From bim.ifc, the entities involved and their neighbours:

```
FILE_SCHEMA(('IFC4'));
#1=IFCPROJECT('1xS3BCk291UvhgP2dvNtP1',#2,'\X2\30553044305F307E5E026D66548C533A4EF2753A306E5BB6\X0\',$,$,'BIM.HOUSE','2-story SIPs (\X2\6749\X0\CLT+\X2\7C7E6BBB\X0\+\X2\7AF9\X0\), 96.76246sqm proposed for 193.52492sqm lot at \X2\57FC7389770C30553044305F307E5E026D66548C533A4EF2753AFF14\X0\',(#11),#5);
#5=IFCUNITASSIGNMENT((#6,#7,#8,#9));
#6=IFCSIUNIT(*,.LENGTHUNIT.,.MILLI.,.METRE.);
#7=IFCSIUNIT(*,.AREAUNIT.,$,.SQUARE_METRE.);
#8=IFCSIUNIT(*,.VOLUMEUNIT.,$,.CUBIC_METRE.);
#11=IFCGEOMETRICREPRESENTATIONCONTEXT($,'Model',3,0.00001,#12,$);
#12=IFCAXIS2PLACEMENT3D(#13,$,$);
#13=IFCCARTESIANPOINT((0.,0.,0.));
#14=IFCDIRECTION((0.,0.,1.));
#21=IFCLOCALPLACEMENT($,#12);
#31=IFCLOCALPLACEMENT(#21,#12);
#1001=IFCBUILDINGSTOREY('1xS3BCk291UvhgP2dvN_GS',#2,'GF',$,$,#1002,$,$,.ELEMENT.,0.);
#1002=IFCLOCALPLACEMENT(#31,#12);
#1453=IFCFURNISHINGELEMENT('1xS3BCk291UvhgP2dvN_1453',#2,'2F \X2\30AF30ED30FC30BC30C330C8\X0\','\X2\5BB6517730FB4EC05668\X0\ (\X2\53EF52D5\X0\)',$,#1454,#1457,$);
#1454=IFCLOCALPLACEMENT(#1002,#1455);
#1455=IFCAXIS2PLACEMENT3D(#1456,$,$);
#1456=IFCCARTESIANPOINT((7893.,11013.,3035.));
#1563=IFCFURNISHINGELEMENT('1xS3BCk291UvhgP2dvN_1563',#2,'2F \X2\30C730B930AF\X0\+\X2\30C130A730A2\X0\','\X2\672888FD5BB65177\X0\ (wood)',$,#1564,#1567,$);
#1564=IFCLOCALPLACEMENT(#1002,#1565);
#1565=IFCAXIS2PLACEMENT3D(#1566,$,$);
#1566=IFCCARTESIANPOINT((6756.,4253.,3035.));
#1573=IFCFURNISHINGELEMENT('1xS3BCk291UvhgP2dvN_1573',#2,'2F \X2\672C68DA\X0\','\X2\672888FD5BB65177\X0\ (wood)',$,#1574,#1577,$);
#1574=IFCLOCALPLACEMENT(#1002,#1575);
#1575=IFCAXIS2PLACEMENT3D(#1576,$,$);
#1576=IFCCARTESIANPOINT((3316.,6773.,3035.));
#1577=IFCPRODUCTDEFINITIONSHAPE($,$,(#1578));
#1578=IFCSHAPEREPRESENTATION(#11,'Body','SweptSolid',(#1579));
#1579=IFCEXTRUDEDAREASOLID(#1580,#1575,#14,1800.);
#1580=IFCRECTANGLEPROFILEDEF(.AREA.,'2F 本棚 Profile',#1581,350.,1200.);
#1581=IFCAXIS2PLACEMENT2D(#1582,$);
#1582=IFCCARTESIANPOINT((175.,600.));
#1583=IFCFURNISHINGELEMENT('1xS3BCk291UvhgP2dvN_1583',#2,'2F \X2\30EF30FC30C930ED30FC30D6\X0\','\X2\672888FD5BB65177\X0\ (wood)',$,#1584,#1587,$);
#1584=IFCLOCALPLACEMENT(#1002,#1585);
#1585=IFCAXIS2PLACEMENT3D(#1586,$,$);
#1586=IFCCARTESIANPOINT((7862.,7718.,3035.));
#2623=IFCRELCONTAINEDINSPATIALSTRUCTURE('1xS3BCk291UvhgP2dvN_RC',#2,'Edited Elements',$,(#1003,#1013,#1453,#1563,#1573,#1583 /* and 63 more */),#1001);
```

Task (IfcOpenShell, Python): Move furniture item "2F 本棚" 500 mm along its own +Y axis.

```python
import ifcopenshell
import ifcopenshell.api.geometry
import ifcopenshell.util.placement
import ifcopenshell.util.unit

model = ifcopenshell.open("bim.ifc")
unit_scale = ifcopenshell.util.unit.calculate_unit_scale(model)

item = model.by_guid("1xS3BCk291UvhgP2dvN_1573")
matrix = ifcopenshell.util.placement.get_local_placement(item.ObjectPlacement)
matrix[:3, 3] += matrix[:3, 1] * 0.5 / unit_scale
ifcopenshell.api.geometry.edit_object_placement(model, product=item, matrix=matrix, is_si=False)

print(ifcopenshell.util.placement.get_local_placement(item.ObjectPlacement).round(3) + 0.0)

model.write("bim-out.ifc")
```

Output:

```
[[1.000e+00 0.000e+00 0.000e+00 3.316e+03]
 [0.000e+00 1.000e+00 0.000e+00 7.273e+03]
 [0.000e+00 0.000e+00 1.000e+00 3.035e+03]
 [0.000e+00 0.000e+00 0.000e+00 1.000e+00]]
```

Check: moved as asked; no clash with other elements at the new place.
